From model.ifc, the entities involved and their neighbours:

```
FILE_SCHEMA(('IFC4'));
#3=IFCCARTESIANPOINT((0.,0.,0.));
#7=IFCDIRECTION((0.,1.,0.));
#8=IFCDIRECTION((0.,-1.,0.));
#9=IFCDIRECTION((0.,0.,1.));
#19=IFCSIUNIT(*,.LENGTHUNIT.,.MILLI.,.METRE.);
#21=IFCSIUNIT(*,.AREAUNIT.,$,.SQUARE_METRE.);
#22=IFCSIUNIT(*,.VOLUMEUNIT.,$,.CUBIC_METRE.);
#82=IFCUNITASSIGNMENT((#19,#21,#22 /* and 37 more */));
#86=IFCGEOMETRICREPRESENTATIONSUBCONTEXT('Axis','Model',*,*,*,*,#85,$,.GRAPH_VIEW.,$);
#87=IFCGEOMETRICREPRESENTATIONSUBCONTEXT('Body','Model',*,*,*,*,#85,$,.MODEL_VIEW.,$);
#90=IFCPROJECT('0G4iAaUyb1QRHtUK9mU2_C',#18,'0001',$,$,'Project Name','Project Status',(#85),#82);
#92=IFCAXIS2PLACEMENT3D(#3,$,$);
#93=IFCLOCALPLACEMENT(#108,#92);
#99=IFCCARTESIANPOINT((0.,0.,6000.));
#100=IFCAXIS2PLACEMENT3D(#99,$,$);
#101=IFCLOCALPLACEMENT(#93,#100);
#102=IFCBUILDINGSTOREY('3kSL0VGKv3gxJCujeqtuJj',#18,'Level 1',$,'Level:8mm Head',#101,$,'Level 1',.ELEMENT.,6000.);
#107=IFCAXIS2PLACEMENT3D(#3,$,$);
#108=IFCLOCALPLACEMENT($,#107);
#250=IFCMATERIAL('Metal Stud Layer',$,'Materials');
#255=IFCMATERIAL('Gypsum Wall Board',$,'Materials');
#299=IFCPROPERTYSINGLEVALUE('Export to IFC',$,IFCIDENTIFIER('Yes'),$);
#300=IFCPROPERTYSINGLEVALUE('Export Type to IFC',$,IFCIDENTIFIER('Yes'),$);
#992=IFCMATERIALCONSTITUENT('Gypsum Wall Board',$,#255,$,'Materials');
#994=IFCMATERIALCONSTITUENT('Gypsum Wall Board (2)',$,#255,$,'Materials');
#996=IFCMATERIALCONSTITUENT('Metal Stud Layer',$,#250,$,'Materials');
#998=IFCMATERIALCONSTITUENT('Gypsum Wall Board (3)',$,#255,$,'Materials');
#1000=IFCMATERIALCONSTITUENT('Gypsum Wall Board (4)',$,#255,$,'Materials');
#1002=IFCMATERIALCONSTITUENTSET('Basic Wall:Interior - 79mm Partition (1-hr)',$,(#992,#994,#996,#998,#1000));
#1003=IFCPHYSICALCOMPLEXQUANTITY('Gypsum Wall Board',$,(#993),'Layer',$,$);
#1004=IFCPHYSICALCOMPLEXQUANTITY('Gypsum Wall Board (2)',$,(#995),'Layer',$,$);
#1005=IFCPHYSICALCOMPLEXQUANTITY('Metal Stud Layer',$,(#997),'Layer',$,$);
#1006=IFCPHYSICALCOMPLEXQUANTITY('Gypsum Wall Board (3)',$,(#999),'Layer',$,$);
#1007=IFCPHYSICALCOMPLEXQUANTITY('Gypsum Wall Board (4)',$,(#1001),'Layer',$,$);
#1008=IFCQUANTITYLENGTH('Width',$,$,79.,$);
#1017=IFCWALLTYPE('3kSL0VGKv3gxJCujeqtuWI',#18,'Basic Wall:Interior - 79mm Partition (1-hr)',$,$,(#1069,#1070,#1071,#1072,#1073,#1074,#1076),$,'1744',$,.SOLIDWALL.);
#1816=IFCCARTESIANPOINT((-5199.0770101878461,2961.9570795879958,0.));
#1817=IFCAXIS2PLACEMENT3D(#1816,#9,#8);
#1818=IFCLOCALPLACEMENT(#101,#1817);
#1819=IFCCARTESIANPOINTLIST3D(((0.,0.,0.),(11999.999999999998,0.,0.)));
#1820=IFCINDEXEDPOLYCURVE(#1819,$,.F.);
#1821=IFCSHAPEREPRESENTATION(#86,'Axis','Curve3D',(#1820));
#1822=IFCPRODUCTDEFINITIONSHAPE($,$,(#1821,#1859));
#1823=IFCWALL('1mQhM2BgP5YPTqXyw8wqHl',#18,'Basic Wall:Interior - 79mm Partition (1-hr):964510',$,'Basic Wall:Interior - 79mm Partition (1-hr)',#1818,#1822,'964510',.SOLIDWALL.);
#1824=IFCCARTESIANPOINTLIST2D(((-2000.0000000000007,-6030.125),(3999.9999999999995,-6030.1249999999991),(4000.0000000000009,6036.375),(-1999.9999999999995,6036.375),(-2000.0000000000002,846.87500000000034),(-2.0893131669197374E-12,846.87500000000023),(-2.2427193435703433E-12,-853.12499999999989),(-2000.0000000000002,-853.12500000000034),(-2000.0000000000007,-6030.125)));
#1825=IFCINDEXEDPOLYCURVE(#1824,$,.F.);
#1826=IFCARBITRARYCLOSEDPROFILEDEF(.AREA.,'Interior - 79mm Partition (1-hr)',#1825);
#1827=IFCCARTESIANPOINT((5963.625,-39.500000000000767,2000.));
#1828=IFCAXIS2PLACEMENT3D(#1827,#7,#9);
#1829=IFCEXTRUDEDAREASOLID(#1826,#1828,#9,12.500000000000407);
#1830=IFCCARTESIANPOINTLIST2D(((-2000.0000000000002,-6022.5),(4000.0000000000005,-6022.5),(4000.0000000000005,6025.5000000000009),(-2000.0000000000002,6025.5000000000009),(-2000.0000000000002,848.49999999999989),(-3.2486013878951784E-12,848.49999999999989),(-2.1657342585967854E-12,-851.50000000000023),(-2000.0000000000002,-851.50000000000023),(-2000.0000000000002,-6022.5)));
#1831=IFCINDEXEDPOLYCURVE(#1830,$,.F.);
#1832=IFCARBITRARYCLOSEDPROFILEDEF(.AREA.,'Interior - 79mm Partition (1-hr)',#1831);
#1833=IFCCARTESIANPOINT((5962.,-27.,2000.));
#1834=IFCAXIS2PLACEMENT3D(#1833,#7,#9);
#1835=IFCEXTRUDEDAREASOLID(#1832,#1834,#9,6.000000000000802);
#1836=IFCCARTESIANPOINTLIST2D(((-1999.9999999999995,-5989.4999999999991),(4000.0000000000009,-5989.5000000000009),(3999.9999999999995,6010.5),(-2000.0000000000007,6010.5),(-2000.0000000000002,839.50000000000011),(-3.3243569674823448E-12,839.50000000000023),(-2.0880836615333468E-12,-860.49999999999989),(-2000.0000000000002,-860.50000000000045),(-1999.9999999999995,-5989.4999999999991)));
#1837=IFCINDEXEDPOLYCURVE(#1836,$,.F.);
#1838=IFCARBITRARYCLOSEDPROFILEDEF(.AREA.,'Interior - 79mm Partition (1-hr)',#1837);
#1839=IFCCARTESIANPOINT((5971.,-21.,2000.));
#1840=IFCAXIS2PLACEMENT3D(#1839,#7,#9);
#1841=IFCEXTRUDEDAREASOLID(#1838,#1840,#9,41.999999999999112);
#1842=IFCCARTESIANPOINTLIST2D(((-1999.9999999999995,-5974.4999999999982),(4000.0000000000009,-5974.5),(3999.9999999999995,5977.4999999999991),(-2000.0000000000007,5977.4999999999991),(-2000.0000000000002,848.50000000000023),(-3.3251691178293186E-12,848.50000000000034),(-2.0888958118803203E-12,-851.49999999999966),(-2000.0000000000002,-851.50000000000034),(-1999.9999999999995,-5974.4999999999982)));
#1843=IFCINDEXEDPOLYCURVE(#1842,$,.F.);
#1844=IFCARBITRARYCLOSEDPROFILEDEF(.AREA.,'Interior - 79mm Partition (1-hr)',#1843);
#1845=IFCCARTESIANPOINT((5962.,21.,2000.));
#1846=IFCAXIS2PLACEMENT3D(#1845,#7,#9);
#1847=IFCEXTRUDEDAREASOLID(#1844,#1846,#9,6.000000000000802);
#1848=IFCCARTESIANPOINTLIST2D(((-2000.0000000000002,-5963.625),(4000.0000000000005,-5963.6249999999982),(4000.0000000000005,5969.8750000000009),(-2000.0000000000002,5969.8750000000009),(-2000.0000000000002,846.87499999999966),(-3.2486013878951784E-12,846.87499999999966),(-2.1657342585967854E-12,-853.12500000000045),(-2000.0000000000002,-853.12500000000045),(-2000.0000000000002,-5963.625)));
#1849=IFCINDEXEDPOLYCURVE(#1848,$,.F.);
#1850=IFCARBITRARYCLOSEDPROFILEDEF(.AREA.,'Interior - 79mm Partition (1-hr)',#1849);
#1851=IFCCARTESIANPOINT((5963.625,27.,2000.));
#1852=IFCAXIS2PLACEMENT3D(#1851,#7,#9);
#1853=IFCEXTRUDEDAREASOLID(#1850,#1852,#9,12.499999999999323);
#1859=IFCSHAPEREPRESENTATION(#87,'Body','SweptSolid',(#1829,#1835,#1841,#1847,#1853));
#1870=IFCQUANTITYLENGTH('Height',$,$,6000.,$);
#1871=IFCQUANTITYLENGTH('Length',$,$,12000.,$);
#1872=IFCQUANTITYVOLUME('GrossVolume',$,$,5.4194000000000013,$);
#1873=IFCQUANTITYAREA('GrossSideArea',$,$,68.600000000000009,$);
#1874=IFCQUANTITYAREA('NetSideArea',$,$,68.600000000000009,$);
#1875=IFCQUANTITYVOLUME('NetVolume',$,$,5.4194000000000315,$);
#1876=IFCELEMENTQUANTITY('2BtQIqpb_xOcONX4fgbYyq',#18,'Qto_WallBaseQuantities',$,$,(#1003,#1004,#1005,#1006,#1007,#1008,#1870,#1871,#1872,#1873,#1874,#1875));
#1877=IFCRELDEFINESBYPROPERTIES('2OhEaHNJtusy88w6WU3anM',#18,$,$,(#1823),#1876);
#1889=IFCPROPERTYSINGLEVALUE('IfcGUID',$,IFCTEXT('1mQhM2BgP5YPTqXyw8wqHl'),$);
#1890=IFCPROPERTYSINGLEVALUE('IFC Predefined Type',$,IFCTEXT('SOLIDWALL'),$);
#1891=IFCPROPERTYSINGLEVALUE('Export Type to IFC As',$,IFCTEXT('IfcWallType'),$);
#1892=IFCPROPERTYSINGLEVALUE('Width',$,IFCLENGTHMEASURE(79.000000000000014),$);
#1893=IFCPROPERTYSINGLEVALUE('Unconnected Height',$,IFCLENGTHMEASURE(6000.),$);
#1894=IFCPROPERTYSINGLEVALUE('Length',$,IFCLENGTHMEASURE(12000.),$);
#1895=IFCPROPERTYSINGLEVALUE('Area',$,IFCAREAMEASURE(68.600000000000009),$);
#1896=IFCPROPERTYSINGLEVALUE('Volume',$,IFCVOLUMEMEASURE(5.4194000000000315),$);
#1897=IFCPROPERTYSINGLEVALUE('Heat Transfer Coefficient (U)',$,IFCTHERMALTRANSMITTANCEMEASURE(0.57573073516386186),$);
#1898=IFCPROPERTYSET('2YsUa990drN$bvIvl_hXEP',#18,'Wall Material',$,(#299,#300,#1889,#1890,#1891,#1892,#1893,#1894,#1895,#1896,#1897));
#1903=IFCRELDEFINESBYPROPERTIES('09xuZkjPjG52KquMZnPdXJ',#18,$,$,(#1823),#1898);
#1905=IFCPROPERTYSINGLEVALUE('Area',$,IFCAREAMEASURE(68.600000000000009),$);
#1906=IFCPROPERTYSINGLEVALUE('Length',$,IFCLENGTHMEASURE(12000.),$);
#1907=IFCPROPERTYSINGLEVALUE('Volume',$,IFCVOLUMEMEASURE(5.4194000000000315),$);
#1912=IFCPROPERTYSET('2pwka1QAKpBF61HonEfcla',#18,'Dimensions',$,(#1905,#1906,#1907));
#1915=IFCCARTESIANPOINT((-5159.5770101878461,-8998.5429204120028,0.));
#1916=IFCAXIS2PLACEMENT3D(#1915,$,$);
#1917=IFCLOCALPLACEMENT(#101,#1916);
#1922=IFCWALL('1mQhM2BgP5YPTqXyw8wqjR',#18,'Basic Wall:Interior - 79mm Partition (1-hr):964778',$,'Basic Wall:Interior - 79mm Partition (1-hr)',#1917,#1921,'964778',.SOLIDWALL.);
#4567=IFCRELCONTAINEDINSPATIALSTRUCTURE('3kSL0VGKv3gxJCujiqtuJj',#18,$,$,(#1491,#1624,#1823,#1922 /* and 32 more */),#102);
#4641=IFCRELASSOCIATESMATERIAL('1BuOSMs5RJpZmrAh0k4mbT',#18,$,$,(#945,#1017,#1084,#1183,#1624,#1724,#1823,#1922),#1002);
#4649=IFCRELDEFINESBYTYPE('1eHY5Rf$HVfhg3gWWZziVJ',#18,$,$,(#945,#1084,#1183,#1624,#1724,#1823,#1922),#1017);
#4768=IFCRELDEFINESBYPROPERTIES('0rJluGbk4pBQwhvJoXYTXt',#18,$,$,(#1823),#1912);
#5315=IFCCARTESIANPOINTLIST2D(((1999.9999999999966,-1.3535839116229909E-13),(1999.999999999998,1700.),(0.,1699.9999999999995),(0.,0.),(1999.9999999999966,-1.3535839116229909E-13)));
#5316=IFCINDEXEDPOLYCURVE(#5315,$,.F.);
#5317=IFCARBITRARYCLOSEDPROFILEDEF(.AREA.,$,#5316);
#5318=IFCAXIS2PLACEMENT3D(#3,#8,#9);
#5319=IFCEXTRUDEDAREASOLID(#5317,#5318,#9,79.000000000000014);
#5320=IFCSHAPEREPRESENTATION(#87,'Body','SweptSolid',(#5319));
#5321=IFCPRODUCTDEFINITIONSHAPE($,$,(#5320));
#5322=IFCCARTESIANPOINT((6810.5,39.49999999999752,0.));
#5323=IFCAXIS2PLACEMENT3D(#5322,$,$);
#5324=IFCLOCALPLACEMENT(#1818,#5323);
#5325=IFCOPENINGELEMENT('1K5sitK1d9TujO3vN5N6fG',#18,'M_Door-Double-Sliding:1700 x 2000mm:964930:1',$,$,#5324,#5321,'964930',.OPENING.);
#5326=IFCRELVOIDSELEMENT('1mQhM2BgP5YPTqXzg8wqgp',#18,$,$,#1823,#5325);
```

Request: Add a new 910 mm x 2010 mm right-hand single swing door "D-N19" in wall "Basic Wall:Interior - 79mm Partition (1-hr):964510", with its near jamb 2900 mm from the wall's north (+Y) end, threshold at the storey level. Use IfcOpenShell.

```python
import numpy as np
import ifcopenshell
import ifcopenshell.api.feature
import ifcopenshell.api.geometry
import ifcopenshell.api.pset
import ifcopenshell.api.root
import ifcopenshell.api.spatial
import ifcopenshell.geom
import ifcopenshell.util.element
import ifcopenshell.util.placement
import ifcopenshell.util.representation
import ifcopenshell.util.shape
import ifcopenshell.util.unit

model = ifcopenshell.open("model.ifc")
unit_scale = ifcopenshell.util.unit.calculate_unit_scale(model)
area_scale = ifcopenshell.util.unit.calculate_unit_scale(model, "AREAUNIT")
volume_scale = ifcopenshell.util.unit.calculate_unit_scale(model, "VOLUMEUNIT")
settings = ifcopenshell.geom.settings()


def volume(element):
    """Net volume in cubic metres, openings subtracted."""
    shape = ifcopenshell.geom.create_shape(settings, element)
    return ifcopenshell.util.shape.get_volume(shape.geometry)


wall = model.by_guid("1mQhM2BgP5YPTqXyw8wqHl")
storey = ifcopenshell.util.element.get_container(wall, ifc_class="IfcBuildingStorey")
context = ifcopenshell.util.representation.get_context(model, "Model", "Body", "MODEL_VIEW")
before = volume(wall)

width, height, from_end, sill = 0.91, 2.01, 2.9, 0.0  # metres

# The wall runs along its own X axis, and the end named is its -X end.
wall_shape = ifcopenshell.geom.create_shape(settings, wall)
x, y, z = ifcopenshell.util.shape.get_vertices(wall_shape.geometry).T
start = x.min() + from_end
face, thickness = float(y.min()), float(y.max() - y.min())
wall_matrix = ifcopenshell.util.placement.get_local_placement(wall.ObjectPlacement)
level = ifcopenshell.util.placement.get_local_placement(storey.ObjectPlacement)[2, 3]


def in_wall(x, y):
    """Placement at x, y metres in the wall's axes, at sill height."""
    matrix = wall_matrix.copy()
    matrix[:, 3] = wall_matrix @ np.array([x / unit_scale, y / unit_scale, 0.0, 1.0])
    matrix[2, 3] = level + sill / unit_scale
    return matrix


# Opening: a box that overshoots both wall faces by 50 mm.
opening = ifcopenshell.api.root.create_entity(model, ifc_class="IfcOpeningElement", predefined_type="OPENING")
box = ifcopenshell.api.geometry.add_wall_representation(
    model, context=context, length=width, height=height, thickness=thickness + 0.1
)
ifcopenshell.api.geometry.assign_representation(model, product=opening, representation=box)
ifcopenshell.api.geometry.edit_object_placement(model, product=opening, matrix=in_wall(start, face - 0.05), is_si=False)
ifcopenshell.api.feature.add_feature(model, feature=opening, element=wall)

door = ifcopenshell.api.root.create_entity(model, ifc_class="IfcDoor", name="D-N19", predefined_type="DOOR")
door.OverallWidth, door.OverallHeight = width / unit_scale, height / unit_scale
door.OperationType = "SINGLE_SWING_RIGHT"
body = ifcopenshell.api.geometry.add_door_representation(
    model,
    context=context,
    overall_width=door.OverallWidth,
    overall_height=door.OverallHeight,
    operation_type="SINGLE_SWING_RIGHT",
    lining_properties={"LiningDepth": thickness / unit_scale, "ThresholdDepth": thickness / unit_scale},
)
ifcopenshell.api.geometry.assign_representation(model, product=door, representation=body)
ifcopenshell.api.spatial.assign_container(model, products=[door], relating_structure=storey)
ifcopenshell.api.feature.add_filling(model, opening=opening, element=door)

# The lining spans the wall, so the door starts at the wall face.
ifcopenshell.api.geometry.edit_object_placement(model, product=door, matrix=in_wall(start, face), is_si=False)

after = volume(wall)

# Update the wall's stored quantities.
qto = model.by_id(ifcopenshell.util.element.get_pset(wall, "Qto_WallBaseQuantities", should_inherit=False)["id"])
ifcopenshell.api.pset.edit_qto(model, qto=qto, properties={
    "NetSideArea": after / thickness / area_scale,
    "NetVolume": after / volume_scale,
})
pset = model.by_id(ifcopenshell.util.element.get_pset(wall, "Wall Material", should_inherit=False)["id"])
ifcopenshell.api.pset.edit_pset(model, pset=pset, properties={
    "Area": model.create_entity("IfcAreaMeasure", after / thickness / area_scale),
    "Volume": model.create_entity("IfcVolumeMeasure", after / volume_scale),
})
pset = model.by_id(ifcopenshell.util.element.get_pset(wall, "Dimensions", should_inherit=False)["id"])
ifcopenshell.api.pset.edit_pset(model, pset=pset, properties={
    "Area": model.create_entity("IfcAreaMeasure", after / thickness / area_scale),
    "Volume": model.create_entity("IfcVolumeMeasure", after / volume_scale),
})

print(f"wall volume {before:.3f} -> {after:.3f} m3")

model.write("model-out.ifc")
```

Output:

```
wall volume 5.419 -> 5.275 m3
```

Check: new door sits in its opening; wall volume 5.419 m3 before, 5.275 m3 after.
